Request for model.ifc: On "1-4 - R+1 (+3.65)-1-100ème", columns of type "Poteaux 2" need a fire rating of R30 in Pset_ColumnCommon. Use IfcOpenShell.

First a look at what the model holds.

```python
import ifcopenshell
import ifcopenshell.util.element

model = ifcopenshell.open("model.ifc")
print(model.schema)
storey = next(s for s in model.by_type("IfcBuildingStorey") if s.Name == "1-4 - R+1 (+3.65)-1-100ème")
columns = [e for e in ifcopenshell.util.element.get_decomposition(storey) if e.is_a("IfcColumn")]
seen = {}
for e in columns:
    element_type = ifcopenshell.util.element.get_type(e)
    key = (element_type.Name if element_type != e and element_type else None, ifcopenshell.util.element.get_pset(e, "Pset_ColumnCommon", "FireRating"))
    seen[key] = seen.get(key, 0) + 1
for (name, value), count in sorted(seen.items(), key=str):
    print(count, "x", name, "|", value)
```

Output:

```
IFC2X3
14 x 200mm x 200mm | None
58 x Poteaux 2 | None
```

```python
import ifcopenshell
import ifcopenshell.api.pset
import ifcopenshell.util.element

model = ifcopenshell.open("model.ifc")

storey = next(s for s in model.by_type("IfcBuildingStorey") if s.Name == "1-4 - R+1 (+3.65)-1-100ème")
columns = [e for e in ifcopenshell.util.element.get_decomposition(storey) if e.is_a("IfcColumn")]

count = 0
for e in columns:
    element_type = ifcopenshell.util.element.get_type(e)
    if element_type in (None, e) or element_type.Name != "Poteaux 2":
        continue
    # add_pset returns the element's existing set when there is one.
    pset = ifcopenshell.api.pset.add_pset(model, product=e, name="Pset_ColumnCommon")
    ifcopenshell.api.pset.edit_pset(model, pset=pset, properties={"FireRating": "R30"})
    count += 1

print(count, "columns updated")

model.write("model_rev.ifc")
```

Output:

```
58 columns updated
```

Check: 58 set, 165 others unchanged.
